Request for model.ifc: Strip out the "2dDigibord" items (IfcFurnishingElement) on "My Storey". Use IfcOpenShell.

First a look at what the model holds.

```python
import ifcopenshell
import ifcopenshell.util.element

model = ifcopenshell.open("model.ifc")
print(model.schema)
storey = next(s for s in model.by_type("IfcBuildingStorey") if s.Name == "My Storey")
furniture = [e for e in ifcopenshell.util.element.get_decomposition(storey) if e.is_a("IfcFurnishingElement")]
seen = {}
for e in furniture:
    element_type = ifcopenshell.util.element.get_type(e)
    name = element_type.Name if element_type not in (None, e) else None
    seen[name] = seen.get(name, 0) + 1
for name, count in sorted(seen.items(), key=str):
    print(count, "x", name)
```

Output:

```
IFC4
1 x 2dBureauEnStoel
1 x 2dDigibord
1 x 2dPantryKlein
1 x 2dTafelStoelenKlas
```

```python
import ifcopenshell
import ifcopenshell.api.root
import ifcopenshell.util.element

model = ifcopenshell.open("model.ifc")

storey = next(s for s in model.by_type("IfcBuildingStorey") if s.Name == "My Storey")
furniture = [e for e in ifcopenshell.util.element.get_decomposition(storey) if e.is_a("IfcFurnishingElement")]
targets = [e for e in furniture if (t := ifcopenshell.util.element.get_type(e)) not in (None, e) and t.Name == "2dDigibord"]

for e in targets:
    ifcopenshell.api.root.remove_product(model, product=e)
print(len(targets), "removed")

model.write("model-out.ifc")
```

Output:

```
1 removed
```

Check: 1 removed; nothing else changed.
